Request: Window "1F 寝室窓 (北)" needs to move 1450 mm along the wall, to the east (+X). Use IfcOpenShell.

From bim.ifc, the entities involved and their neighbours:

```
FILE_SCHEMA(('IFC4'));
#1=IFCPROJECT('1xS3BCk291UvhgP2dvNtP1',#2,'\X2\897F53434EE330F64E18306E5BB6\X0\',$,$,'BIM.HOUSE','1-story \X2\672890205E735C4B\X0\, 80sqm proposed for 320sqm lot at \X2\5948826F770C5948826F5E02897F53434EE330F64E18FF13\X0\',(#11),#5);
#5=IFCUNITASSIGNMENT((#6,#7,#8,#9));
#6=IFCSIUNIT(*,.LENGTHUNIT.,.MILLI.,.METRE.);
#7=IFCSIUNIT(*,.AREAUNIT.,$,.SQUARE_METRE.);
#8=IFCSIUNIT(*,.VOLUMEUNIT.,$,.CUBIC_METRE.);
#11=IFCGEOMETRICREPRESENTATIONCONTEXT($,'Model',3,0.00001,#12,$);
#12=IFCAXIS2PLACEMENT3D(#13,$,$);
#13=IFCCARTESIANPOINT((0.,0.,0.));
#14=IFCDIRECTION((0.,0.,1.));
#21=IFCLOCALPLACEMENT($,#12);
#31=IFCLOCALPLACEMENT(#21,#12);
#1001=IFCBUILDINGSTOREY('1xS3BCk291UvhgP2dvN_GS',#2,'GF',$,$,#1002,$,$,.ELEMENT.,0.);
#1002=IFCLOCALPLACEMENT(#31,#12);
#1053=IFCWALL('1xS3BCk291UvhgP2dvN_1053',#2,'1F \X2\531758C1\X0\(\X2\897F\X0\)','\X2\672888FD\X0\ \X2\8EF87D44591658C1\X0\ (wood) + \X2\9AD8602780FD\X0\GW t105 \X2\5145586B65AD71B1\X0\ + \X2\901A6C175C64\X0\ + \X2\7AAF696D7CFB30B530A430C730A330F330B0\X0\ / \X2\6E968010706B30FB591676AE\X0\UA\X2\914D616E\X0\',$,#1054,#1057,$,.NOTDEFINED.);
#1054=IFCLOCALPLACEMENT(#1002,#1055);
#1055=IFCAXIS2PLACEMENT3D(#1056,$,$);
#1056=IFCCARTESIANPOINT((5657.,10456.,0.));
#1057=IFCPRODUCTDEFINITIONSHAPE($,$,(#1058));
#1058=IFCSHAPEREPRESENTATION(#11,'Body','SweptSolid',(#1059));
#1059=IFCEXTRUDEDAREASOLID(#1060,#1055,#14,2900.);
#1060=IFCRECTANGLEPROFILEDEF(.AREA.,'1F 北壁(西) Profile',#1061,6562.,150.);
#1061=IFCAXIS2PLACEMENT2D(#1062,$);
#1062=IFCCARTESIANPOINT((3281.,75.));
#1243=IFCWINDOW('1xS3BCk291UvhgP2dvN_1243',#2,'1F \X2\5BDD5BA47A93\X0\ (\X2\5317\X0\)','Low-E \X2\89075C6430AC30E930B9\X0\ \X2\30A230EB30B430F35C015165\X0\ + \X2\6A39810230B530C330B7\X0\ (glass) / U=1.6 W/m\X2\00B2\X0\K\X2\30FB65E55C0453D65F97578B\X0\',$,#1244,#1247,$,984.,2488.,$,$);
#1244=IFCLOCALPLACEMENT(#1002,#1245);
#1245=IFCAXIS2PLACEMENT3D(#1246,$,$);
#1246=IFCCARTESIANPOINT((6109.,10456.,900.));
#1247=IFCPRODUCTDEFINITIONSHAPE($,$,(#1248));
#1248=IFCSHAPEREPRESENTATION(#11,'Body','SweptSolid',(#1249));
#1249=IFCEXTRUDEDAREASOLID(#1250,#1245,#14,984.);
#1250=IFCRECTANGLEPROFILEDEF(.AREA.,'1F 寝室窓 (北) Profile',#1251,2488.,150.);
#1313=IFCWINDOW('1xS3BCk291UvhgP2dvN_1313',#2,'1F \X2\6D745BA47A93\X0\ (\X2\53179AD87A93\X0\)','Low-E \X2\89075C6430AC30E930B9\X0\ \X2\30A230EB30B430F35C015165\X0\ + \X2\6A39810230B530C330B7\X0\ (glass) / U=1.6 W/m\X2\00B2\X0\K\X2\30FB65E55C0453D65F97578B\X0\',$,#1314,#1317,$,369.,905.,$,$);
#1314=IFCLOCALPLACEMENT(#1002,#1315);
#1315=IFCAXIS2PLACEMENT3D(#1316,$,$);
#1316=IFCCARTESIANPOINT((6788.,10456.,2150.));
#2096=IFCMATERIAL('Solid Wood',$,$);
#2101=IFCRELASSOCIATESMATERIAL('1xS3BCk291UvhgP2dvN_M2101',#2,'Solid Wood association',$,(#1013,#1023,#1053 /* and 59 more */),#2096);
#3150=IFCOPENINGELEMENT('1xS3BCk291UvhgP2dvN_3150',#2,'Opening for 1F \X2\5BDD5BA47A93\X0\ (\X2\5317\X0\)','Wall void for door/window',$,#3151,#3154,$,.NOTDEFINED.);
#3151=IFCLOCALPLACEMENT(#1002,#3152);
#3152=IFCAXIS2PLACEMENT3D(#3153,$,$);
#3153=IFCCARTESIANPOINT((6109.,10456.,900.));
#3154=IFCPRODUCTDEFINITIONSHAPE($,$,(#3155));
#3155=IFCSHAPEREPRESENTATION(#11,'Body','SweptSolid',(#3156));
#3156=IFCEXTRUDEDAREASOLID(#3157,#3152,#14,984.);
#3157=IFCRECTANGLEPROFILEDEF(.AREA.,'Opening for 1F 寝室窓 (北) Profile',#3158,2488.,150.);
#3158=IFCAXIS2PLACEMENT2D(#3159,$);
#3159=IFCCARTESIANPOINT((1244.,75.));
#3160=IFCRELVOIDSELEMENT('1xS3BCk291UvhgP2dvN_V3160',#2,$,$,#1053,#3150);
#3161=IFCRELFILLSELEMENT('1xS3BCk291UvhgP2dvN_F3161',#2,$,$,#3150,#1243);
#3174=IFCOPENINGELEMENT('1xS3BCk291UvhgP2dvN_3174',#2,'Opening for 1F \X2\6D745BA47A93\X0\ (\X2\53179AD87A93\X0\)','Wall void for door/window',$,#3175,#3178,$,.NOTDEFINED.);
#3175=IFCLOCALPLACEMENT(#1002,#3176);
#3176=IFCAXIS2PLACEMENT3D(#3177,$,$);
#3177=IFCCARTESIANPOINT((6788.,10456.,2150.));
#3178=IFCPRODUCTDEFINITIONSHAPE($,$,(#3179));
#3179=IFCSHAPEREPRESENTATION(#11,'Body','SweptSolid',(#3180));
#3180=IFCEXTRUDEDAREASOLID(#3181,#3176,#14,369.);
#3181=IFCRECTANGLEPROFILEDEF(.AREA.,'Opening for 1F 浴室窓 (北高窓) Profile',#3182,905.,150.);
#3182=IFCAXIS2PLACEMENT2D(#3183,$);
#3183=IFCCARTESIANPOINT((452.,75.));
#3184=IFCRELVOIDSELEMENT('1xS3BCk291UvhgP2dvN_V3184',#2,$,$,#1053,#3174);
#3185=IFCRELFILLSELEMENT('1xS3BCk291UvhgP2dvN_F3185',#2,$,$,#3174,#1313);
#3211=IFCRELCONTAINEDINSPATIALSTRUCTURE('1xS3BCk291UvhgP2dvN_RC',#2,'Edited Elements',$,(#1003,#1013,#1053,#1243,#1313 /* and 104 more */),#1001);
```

```python
import ifcopenshell
import ifcopenshell.api.geometry
import ifcopenshell.util.placement
import ifcopenshell.util.unit

model = ifcopenshell.open("bim.ifc")
unit_scale = ifcopenshell.util.unit.calculate_unit_scale(model)

window = model.by_guid("1xS3BCk291UvhgP2dvN_1243")
opening = window.FillsVoids[0].RelatingOpeningElement
wall = opening.VoidsElements[0].RelatingBuildingElement

wall_matrix = ifcopenshell.util.placement.get_local_placement(wall.ObjectPlacement)
shift = wall_matrix[:3, 0] * 1.45 / unit_scale
before = ifcopenshell.util.placement.get_local_placement(window.ObjectPlacement)[:3, 3].copy()

# The window is not placed relative to its opening, so move both.
for product in (opening, window):
    matrix = ifcopenshell.util.placement.get_local_placement(product.ObjectPlacement)
    matrix[:3, 3] += shift
    ifcopenshell.api.geometry.edit_object_placement(model, product=product, matrix=matrix, is_si=False)

after = ifcopenshell.util.placement.get_local_placement(window.ObjectPlacement)[:3, 3]
print("window moved by", (after - before).round(3) + 0.0)

model.write("bim-out.ifc")
```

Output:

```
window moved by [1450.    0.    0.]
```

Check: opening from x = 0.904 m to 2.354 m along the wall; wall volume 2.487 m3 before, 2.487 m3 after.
